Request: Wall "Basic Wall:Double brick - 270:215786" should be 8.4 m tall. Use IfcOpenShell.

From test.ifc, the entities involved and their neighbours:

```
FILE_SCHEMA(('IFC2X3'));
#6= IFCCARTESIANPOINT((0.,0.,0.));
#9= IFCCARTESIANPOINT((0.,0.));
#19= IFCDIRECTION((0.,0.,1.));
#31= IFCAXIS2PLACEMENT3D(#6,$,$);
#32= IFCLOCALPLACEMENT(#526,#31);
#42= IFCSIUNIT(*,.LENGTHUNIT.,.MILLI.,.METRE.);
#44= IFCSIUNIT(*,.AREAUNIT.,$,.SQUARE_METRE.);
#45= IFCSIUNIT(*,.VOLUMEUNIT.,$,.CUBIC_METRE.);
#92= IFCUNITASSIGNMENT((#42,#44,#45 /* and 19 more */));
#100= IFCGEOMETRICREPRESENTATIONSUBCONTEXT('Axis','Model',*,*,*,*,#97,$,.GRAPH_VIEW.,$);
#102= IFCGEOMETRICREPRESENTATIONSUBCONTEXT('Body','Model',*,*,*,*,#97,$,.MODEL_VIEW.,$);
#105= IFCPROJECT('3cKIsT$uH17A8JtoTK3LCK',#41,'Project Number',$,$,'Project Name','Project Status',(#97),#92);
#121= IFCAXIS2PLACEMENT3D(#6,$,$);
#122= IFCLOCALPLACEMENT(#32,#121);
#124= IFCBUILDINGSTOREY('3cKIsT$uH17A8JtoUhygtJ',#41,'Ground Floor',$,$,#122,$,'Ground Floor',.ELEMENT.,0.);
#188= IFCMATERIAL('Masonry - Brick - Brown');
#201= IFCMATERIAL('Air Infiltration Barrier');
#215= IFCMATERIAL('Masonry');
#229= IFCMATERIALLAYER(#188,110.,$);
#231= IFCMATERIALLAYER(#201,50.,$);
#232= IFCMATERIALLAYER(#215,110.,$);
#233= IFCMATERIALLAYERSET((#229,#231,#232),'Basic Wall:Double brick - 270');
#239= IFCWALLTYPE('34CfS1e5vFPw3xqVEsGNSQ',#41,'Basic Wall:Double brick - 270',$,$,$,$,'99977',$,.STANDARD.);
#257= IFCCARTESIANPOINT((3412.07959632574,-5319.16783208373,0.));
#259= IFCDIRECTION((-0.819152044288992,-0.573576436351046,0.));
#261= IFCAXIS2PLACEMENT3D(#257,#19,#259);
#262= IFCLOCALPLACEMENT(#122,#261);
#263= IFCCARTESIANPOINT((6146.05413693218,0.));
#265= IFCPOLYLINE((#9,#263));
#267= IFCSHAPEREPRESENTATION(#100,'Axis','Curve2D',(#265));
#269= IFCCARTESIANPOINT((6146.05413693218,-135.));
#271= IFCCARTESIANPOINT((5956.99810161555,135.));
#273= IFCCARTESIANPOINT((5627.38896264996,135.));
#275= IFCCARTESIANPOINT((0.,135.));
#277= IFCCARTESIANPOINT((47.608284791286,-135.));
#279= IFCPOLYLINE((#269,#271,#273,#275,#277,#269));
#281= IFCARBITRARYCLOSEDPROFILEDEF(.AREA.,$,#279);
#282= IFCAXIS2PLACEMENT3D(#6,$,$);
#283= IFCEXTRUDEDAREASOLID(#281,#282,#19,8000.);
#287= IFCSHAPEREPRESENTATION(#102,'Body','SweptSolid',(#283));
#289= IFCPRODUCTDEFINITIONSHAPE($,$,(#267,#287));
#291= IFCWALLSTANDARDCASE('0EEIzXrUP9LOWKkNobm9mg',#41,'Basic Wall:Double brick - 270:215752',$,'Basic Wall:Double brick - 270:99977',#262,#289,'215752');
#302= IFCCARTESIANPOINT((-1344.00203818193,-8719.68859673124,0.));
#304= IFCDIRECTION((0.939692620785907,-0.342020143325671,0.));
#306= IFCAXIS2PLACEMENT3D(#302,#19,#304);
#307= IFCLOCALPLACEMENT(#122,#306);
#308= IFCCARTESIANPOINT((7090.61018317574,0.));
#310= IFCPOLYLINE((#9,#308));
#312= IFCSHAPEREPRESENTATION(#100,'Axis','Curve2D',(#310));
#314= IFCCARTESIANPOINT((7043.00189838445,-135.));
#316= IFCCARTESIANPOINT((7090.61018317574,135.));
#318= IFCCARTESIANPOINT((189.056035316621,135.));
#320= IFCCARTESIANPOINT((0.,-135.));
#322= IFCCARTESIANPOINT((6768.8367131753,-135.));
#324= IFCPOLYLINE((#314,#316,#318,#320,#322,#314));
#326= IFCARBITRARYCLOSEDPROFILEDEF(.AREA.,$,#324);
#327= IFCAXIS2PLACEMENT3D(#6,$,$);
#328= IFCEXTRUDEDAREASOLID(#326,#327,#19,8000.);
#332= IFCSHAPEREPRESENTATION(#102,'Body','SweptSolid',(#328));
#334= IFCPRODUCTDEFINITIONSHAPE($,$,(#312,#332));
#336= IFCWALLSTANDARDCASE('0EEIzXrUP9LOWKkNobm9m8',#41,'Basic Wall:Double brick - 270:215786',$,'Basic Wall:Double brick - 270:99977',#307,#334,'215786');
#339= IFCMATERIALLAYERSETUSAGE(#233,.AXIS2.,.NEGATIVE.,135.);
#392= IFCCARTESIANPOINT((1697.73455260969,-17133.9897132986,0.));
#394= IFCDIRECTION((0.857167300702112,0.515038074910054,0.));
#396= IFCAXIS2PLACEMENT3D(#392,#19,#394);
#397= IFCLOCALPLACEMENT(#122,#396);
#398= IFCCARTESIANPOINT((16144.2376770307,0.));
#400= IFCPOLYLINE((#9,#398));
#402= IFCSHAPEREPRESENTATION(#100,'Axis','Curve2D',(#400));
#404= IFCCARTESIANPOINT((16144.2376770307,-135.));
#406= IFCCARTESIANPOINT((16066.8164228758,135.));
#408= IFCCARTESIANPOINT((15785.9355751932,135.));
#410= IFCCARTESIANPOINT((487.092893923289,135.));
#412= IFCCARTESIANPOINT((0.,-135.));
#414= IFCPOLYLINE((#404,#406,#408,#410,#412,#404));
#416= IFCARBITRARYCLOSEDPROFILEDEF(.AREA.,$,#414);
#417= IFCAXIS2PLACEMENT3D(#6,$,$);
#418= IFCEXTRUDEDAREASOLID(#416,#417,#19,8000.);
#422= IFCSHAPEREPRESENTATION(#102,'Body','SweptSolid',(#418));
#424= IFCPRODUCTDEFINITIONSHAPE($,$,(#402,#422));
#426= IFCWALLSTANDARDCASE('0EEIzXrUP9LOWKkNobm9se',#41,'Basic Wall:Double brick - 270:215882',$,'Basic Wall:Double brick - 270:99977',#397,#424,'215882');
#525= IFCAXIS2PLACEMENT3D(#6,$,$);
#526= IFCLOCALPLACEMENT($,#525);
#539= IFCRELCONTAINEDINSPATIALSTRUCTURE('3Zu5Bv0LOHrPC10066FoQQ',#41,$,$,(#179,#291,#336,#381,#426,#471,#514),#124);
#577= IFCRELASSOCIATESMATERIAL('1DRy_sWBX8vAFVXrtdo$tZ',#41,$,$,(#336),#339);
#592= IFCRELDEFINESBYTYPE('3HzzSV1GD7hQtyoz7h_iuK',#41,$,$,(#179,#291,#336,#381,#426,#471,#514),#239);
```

```python
import ifcopenshell
import ifcopenshell.geom
import ifcopenshell.util.representation
import ifcopenshell.util.shape

model = ifcopenshell.open("test.ifc")
settings = ifcopenshell.geom.settings()


def volume(element):
    """Net volume in cubic metres, openings subtracted."""
    shape = ifcopenshell.geom.create_shape(settings, element)
    return ifcopenshell.util.shape.get_volume(shape.geometry)


wall = model.by_guid("0EEIzXrUP9LOWKkNobm9m8")
before = volume(wall)

body = ifcopenshell.util.representation.get_representation(wall, "Model", "Body")
solid = body.Items[0]
old_height = solid.Depth
solid.Depth = 8400.0
after = volume(wall)

print(f"height {old_height:g} -> {solid.Depth:g}, volume {before:.3f} -> {after:.3f} m3")

model.write("test_v2.ifc")
```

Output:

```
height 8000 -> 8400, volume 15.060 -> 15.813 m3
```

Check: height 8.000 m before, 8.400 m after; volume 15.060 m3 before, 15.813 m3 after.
